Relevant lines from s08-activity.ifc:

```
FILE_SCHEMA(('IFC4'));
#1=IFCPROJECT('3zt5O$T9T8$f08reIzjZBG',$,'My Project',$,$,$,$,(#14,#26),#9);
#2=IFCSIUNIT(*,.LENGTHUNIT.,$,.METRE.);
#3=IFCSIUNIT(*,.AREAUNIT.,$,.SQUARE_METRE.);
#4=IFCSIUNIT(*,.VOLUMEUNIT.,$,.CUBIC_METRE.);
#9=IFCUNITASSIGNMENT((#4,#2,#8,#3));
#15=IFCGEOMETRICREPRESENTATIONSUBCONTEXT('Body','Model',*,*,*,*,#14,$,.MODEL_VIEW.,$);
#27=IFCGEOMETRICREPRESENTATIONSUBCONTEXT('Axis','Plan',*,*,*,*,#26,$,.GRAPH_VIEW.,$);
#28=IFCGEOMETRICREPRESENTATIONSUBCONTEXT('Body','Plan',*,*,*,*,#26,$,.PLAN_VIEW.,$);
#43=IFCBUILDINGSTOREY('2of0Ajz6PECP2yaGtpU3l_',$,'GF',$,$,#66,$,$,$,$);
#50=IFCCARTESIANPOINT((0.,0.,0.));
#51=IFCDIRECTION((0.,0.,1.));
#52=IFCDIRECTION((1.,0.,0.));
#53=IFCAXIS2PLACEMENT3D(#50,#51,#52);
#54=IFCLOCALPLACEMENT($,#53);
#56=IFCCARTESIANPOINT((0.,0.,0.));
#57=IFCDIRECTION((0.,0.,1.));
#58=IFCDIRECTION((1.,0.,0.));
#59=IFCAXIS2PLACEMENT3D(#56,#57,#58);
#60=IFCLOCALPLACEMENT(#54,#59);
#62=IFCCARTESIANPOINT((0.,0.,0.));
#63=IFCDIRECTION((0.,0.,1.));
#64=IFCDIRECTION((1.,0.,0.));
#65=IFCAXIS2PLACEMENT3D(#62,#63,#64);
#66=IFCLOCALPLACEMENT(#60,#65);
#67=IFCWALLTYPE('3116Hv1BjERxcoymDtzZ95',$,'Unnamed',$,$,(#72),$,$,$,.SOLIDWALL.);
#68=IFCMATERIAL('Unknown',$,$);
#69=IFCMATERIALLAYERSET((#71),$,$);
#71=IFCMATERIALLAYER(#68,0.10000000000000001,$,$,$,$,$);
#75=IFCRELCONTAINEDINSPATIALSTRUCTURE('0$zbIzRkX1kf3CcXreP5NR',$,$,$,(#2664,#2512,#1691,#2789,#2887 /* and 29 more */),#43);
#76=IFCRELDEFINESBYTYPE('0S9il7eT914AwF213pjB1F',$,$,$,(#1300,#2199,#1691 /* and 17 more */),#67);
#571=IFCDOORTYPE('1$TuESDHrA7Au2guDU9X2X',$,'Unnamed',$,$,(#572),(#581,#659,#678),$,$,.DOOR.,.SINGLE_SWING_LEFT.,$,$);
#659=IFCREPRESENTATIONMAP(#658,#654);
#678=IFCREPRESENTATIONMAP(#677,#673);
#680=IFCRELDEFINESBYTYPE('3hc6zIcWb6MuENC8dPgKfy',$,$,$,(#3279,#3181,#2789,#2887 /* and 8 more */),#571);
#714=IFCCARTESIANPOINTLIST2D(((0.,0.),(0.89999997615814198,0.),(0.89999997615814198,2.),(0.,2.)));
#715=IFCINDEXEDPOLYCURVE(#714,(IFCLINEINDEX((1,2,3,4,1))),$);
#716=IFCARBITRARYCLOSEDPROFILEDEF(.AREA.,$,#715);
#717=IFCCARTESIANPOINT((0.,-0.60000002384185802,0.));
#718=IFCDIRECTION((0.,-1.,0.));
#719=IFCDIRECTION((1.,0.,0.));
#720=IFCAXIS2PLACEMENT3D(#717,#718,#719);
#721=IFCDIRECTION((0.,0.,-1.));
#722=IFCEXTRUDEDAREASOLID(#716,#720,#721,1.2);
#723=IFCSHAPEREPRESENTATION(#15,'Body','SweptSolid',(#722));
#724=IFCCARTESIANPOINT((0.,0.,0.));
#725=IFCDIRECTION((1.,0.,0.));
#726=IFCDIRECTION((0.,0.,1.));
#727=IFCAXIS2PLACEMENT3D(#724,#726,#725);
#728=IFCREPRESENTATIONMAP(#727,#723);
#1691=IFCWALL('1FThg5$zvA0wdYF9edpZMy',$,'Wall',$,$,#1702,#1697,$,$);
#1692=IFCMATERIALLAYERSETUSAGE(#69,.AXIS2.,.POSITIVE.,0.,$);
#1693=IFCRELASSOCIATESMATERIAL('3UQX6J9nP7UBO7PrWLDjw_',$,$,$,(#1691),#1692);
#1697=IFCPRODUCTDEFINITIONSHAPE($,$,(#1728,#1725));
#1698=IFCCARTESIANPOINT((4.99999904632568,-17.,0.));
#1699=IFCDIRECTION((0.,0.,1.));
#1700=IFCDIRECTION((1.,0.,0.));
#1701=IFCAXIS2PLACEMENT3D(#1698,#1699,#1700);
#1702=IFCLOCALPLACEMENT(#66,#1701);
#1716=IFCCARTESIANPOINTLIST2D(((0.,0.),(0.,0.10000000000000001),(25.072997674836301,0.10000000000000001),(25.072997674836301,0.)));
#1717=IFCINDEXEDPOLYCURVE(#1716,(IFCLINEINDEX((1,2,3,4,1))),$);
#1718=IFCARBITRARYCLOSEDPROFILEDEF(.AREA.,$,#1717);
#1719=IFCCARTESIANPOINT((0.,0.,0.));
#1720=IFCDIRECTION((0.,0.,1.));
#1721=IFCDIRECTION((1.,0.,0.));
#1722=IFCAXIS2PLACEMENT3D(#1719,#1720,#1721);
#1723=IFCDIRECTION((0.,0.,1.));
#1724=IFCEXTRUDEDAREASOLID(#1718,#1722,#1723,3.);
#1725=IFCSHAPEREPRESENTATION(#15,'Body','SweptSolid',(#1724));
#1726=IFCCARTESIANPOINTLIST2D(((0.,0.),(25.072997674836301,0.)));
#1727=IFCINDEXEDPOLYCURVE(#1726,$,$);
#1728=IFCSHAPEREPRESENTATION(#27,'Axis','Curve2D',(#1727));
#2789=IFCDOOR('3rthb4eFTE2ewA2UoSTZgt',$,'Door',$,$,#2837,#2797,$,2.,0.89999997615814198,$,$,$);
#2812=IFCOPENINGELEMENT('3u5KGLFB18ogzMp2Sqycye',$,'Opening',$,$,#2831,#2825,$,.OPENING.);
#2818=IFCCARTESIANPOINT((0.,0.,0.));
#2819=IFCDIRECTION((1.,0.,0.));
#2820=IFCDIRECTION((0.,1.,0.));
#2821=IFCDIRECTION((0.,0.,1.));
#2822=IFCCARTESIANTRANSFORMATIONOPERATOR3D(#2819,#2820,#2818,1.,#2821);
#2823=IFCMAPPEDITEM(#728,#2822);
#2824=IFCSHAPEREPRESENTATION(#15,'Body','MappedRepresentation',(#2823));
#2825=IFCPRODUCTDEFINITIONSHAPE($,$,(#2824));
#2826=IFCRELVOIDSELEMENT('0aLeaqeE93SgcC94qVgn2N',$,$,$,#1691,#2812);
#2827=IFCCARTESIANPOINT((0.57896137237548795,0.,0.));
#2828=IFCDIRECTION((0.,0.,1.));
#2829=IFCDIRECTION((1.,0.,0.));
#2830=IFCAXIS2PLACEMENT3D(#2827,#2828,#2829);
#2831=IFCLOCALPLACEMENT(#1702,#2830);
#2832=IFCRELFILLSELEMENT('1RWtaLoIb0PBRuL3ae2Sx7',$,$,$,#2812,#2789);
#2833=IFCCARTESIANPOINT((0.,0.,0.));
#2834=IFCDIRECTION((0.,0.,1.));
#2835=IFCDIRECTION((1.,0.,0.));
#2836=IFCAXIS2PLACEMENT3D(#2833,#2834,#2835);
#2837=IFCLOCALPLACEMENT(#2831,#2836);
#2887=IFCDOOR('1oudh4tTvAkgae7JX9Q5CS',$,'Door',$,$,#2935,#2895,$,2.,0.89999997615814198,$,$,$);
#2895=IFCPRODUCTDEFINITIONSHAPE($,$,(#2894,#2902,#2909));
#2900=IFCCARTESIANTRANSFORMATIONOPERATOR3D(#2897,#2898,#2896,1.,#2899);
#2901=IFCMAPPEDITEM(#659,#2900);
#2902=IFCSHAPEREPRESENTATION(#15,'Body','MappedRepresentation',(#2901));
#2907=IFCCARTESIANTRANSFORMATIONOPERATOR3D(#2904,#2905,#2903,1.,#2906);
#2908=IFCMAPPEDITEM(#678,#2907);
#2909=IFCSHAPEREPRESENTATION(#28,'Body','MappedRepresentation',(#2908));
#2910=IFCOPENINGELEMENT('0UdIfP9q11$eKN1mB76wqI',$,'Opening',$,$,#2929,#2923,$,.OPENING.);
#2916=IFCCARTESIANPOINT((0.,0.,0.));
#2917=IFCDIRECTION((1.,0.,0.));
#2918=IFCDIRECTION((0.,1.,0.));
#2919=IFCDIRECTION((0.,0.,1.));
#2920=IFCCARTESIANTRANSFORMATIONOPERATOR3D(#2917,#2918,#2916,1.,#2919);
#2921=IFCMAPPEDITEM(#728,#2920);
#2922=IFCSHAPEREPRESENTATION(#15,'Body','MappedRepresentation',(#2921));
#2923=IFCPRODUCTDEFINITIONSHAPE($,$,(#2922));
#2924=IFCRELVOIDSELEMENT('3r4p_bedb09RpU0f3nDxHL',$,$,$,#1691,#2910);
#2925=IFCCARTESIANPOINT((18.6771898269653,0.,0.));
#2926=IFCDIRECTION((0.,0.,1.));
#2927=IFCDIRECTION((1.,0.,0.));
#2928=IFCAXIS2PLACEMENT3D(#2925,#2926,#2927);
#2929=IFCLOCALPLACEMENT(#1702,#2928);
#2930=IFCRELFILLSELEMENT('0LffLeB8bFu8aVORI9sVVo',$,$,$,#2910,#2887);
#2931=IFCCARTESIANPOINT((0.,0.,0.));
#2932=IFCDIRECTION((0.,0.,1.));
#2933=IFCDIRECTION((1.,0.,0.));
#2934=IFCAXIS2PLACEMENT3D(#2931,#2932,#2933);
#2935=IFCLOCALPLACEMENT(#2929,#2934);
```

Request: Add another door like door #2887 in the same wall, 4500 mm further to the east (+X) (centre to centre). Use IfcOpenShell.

```python
import ifcopenshell
import ifcopenshell.api.feature
import ifcopenshell.api.geometry
import ifcopenshell.api.root
import ifcopenshell.geom
import ifcopenshell.util.element
import ifcopenshell.util.placement
import ifcopenshell.util.shape

model = ifcopenshell.open("s08-activity.ifc")
settings = ifcopenshell.geom.settings()


def volume(element):
    """Net volume in cubic metres, openings subtracted."""
    shape = ifcopenshell.geom.create_shape(settings, element)
    return ifcopenshell.util.shape.get_volume(shape.geometry)


door = model.by_guid("1oudh4tTvAkgae7JX9Q5CS")
opening = door.FillsVoids[0].RelatingOpeningElement
wall = opening.VoidsElements[0].RelatingBuildingElement
before = volume(wall)
shift = ifcopenshell.util.placement.get_local_placement(wall.ObjectPlacement)[:3, 0] * 4.5

# copy_class copies the void relationship, type, container and properties, but no geometry.
new_opening = ifcopenshell.api.root.copy_class(model, product=opening)
new_opening.Representation = ifcopenshell.util.element.copy_deep(
    model, opening.Representation, exclude=["IfcGeometricRepresentationContext", "IfcRepresentationMap"]
)
new_door = ifcopenshell.api.root.copy_class(model, product=door)
new_door.Representation = ifcopenshell.util.element.copy_deep(
    model, door.Representation, exclude=["IfcGeometricRepresentationContext", "IfcRepresentationMap"]
)
ifcopenshell.api.feature.add_filling(model, opening=new_opening, element=new_door)

for old, new in ((opening, new_opening), (door, new_door)):
    matrix = ifcopenshell.util.placement.get_local_placement(old.ObjectPlacement)
    matrix[:3, 3] += shift
    ifcopenshell.api.geometry.edit_object_placement(model, product=new, matrix=matrix, is_si=False)

after = volume(wall)

print(f"wall volume {before:.3f} -> {after:.3f} m3")

model.write("s08-activity_edited.ifc")
```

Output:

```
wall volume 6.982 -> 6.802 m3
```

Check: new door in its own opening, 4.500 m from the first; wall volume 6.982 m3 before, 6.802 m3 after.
